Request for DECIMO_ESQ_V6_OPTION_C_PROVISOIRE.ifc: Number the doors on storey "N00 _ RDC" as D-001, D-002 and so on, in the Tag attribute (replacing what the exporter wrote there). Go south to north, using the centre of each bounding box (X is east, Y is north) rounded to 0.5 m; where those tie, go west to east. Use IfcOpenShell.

First a look at what the model holds.

```python
import ifcopenshell
import ifcopenshell.util.element
import ifcopenshell.util.placement

model = ifcopenshell.open("DECIMO_ESQ_V6_OPTION_C_PROVISOIRE.ifc")
print(model.schema)
storey = next(s for s in model.by_type("IfcBuildingStorey") if s.Name == "N00 _ RDC")
doors = [e for e in ifcopenshell.util.element.get_decomposition(storey) if e.is_a("IfcDoor")]
for e in sorted(doors, key=lambda e: e.id()):
    origin = ifcopenshell.util.placement.get_local_placement(e.ObjectPlacement)[:3, 3]
    print(e.id(), e.Tag, e.Name, origin.round(2) + 0.0, sep=" | ")
```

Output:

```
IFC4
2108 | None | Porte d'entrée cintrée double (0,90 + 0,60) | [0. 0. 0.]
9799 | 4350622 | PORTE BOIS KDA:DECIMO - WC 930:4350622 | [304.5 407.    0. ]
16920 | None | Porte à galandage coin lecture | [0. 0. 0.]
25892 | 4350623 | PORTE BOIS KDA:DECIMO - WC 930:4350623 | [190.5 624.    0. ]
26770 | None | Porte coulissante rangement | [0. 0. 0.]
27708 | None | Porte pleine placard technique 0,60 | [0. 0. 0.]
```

```python
import ifcopenshell
import ifcopenshell.geom
import ifcopenshell.util.element
import ifcopenshell.util.shape

model = ifcopenshell.open("DECIMO_ESQ_V6_OPTION_C_PROVISOIRE.ifc")
settings = ifcopenshell.geom.settings()
settings.set("use-world-coords", True)


def centre(element):
    shape = ifcopenshell.geom.create_shape(settings, element)
    return ifcopenshell.util.shape.get_bbox_centroid(shape.geometry)


storey = next(s for s in model.by_type("IfcBuildingStorey") if s.Name == "N00 _ RDC")
doors = [e for e in ifcopenshell.util.element.get_decomposition(storey) if e.is_a("IfcDoor")]

# Insertion points can sit at a corner or the storey origin, so sort by the geometry (in metres).
centres = {e: centre(e) for e in doors}
doors.sort(key=lambda e: (round(centres[e][1] / 0.5), centres[e][0]))

for i, e in enumerate(doors, start=1):
    number = f"D-0{i:02d}"
    e.Tag = number
    print(e.id(), number)

model.write("DECIMO_ESQ_V6_OPTION_C_PROVISOIRE_rev.ifc")
```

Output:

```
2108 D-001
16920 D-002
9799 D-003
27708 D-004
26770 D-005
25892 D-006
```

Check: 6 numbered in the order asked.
